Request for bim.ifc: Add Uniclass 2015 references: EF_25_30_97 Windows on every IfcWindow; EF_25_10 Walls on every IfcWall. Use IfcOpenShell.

First a look at what the model holds.

```python
import ifcopenshell

model = ifcopenshell.open("bim.ifc")
print(model.schema)
print("classifications:", [c.Name for c in model.by_type("IfcClassification")])
for ifc_class in ("IfcDoor", "IfcRoof", "IfcStair", "IfcWall", "IfcWindow"):
    print(ifc_class, len(model.by_type(ifc_class)))
```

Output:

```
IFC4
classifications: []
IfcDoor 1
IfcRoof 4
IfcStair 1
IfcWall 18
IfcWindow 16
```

```python
import ifcopenshell
import ifcopenshell.api.classification

model = ifcopenshell.open("bim.ifc")

system = ifcopenshell.api.classification.add_classification(model, classification="Uniclass 2015")

codes = {
    "IfcWindow": ("EF_25_30_97", "Windows"),
    "IfcWall": ("EF_25_10", "Walls"),
}
for ifc_class, (code, name) in codes.items():
    products = model.by_type(ifc_class)
    ifcopenshell.api.classification.add_reference(
        model, products=products, classification=system, identification=code, name=name
    )
    print(code, len(products))

model.write("bim_edited.ifc")
```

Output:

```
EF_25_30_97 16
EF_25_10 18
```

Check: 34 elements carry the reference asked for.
